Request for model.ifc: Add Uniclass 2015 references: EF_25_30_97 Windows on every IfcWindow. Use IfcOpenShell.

First a look at what the model holds.

```python
import ifcopenshell

model = ifcopenshell.open("model.ifc")
print(model.schema)
print("classifications:", [c.Name for c in model.by_type("IfcClassification")])
for ifc_class in ("IfcDoor", "IfcRoof", "IfcStair", "IfcWall", "IfcWindow"):
    print(ifc_class, len(model.by_type(ifc_class)))
```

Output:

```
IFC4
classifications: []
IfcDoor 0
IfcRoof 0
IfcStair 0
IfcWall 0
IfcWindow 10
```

```python
import ifcopenshell
import ifcopenshell.api.classification

model = ifcopenshell.open("model.ifc")

system = ifcopenshell.api.classification.add_classification(model, classification="Uniclass 2015")

codes = {
    "IfcWindow": ("EF_25_30_97", "Windows"),
}
for ifc_class, (code, name) in codes.items():
    products = model.by_type(ifc_class)
    ifcopenshell.api.classification.add_reference(
        model, products=products, classification=system, identification=code, name=name
    )
    print(code, len(products))

model.write("model_edited.ifc")
```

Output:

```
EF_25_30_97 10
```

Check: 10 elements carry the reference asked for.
